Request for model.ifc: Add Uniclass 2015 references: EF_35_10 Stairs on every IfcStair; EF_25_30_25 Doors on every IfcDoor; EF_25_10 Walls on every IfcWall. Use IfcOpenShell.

First a look at what the model holds.

```python
import ifcopenshell

model = ifcopenshell.open("model.ifc")
print(model.schema)
print("classifications:", [c.Name for c in model.by_type("IfcClassification")])
for ifc_class in ("IfcDoor", "IfcRoof", "IfcStair", "IfcWall", "IfcWindow"):
    print(ifc_class, len(model.by_type(ifc_class)))
```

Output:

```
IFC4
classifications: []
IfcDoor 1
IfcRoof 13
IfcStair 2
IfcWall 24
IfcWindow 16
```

```python
import ifcopenshell
import ifcopenshell.api.classification

model = ifcopenshell.open("model.ifc")

system = ifcopenshell.api.classification.add_classification(model, classification="Uniclass 2015")

codes = {
    "IfcStair": ("EF_35_10", "Stairs"),
    "IfcDoor": ("EF_25_30_25", "Doors"),
    "IfcWall": ("EF_25_10", "Walls"),
}
for ifc_class, (code, name) in codes.items():
    products = model.by_type(ifc_class)
    ifcopenshell.api.classification.add_reference(
        model, products=products, classification=system, identification=code, name=name
    )
    print(code, len(products))

model.write("model_rev.ifc")
```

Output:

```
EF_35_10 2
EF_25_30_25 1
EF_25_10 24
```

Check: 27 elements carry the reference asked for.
